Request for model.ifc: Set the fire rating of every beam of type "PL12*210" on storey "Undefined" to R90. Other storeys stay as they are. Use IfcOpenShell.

First a look at what the model holds.

```python
import ifcopenshell
import ifcopenshell.util.element

model = ifcopenshell.open("model.ifc")
print(model.schema)
storey = next(s for s in model.by_type("IfcBuildingStorey") if s.Name == "Undefined")
beams = [e for e in ifcopenshell.util.element.get_decomposition(storey) if e.is_a("IfcBeam")]
seen = {}
for e in beams:
    element_type = ifcopenshell.util.element.get_type(e)
    key = (element_type.Name if element_type != e and element_type else None, ifcopenshell.util.element.get_pset(e, "Pset_BeamCommon", "FireRating"))
    seen[key] = seen.get(key, 0) + 1
for (name, value), count in sorted(seen.items(), key=str):
    print(count, "x", name, "|", value)
```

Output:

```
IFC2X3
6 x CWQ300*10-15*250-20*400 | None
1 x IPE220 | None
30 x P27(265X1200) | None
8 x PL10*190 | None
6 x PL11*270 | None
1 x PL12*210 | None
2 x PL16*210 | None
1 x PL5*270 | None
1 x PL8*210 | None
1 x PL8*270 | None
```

```python
import ifcopenshell
import ifcopenshell.api.pset
import ifcopenshell.util.element

model = ifcopenshell.open("model.ifc")

storey = next(s for s in model.by_type("IfcBuildingStorey") if s.Name == "Undefined")
beams = [e for e in ifcopenshell.util.element.get_decomposition(storey) if e.is_a("IfcBeam")]

count = 0
for e in beams:
    element_type = ifcopenshell.util.element.get_type(e)
    if element_type in (None, e) or element_type.Name != "PL12*210":
        continue
    found = ifcopenshell.util.element.get_pset(e, "Pset_BeamCommon", should_inherit=False)
    if found:
        pset = model.by_id(found["id"])
        if len(ifcopenshell.util.element.get_elements_by_pset(pset)) > 1:
            pset = ifcopenshell.api.pset.unshare_pset(model, products=[e], pset=pset)[0]
    else:
        pset = ifcopenshell.api.pset.add_pset(model, product=e, name="Pset_BeamCommon")
    ifcopenshell.api.pset.edit_pset(model, pset=pset, properties={"FireRating": "R90"})
    count += 1

print(count, "beams updated")

model.write("model_edited.ifc")
```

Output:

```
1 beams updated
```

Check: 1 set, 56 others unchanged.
